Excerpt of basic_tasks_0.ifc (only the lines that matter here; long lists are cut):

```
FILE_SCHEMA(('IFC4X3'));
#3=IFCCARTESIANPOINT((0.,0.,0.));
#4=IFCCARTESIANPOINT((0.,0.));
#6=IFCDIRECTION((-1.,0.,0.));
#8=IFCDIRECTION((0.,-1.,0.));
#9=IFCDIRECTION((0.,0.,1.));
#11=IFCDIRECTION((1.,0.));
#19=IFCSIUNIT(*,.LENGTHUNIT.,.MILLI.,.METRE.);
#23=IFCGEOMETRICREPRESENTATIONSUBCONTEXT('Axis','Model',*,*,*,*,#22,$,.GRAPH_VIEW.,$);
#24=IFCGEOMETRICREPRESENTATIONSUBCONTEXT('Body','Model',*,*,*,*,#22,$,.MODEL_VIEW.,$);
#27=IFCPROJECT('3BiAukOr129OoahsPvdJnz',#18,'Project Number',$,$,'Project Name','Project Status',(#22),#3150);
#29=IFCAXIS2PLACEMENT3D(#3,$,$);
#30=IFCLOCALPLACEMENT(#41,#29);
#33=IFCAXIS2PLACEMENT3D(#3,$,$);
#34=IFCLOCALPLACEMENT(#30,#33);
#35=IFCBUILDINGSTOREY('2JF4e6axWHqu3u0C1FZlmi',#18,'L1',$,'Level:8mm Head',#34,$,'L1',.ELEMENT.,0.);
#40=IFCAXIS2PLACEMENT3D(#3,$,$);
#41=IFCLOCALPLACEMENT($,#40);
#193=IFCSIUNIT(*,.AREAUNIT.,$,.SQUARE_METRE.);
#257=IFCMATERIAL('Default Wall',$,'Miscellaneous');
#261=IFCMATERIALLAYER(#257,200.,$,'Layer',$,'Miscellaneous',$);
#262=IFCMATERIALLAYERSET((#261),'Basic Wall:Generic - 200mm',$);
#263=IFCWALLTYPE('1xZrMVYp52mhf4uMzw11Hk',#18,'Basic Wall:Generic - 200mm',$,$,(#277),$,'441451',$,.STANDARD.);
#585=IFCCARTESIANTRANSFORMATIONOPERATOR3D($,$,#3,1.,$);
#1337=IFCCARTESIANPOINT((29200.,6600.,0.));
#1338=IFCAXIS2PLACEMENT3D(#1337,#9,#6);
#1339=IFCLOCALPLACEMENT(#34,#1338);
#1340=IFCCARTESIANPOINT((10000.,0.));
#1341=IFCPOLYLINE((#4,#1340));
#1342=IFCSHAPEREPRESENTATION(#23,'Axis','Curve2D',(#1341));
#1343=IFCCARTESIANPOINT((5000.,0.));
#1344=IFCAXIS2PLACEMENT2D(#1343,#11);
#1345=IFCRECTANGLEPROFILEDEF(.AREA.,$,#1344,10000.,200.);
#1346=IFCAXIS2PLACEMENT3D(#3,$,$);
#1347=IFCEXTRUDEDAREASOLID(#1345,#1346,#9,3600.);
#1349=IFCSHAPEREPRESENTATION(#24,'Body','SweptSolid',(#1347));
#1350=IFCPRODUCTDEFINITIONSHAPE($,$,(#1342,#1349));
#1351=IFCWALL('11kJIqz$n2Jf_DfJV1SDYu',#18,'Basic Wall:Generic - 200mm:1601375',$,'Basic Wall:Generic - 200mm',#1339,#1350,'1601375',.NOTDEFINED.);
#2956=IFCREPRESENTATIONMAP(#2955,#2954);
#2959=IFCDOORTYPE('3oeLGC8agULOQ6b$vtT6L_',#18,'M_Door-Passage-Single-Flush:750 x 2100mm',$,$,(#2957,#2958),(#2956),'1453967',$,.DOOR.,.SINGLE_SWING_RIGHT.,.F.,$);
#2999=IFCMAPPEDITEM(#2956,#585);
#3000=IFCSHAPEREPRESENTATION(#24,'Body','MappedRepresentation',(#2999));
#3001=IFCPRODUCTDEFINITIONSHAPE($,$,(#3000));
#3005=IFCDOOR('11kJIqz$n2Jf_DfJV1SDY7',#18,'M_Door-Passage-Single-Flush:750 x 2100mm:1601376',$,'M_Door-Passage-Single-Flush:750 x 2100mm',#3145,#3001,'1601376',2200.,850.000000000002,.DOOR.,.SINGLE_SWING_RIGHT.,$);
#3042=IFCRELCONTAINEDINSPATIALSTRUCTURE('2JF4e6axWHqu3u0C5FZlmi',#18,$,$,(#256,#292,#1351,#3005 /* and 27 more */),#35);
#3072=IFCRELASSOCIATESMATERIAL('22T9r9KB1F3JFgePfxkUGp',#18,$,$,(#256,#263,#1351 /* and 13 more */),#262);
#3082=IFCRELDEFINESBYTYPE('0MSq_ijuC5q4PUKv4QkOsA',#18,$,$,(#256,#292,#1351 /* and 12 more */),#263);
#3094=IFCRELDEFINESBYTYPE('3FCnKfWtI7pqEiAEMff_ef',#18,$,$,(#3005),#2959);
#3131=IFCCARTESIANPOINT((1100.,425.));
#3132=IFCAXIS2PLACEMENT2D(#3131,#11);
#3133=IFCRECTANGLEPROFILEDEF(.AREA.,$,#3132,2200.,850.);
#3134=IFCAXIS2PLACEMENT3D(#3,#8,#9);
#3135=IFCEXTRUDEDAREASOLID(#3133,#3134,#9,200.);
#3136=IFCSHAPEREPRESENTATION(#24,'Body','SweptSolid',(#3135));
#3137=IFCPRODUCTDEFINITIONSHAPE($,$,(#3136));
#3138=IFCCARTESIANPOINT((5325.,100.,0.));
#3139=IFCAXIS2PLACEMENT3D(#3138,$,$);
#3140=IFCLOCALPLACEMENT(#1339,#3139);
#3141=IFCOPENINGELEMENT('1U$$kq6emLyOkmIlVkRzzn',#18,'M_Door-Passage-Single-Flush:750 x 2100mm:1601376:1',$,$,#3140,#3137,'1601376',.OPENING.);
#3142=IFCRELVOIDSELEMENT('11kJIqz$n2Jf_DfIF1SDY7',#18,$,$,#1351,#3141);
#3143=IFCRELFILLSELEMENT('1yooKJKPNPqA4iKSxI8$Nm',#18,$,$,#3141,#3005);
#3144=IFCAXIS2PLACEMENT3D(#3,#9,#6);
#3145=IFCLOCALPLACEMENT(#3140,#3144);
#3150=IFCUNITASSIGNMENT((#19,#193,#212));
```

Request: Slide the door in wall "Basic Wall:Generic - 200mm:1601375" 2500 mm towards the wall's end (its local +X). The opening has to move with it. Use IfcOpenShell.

```python
import ifcopenshell
import ifcopenshell.api.geometry
import ifcopenshell.util.placement
import ifcopenshell.util.unit

model = ifcopenshell.open("basic_tasks_0.ifc")
unit_scale = ifcopenshell.util.unit.calculate_unit_scale(model)

door = model.by_guid("11kJIqz$n2Jf_DfJV1SDY7")
opening = door.FillsVoids[0].RelatingOpeningElement
wall = opening.VoidsElements[0].RelatingBuildingElement

wall_matrix = ifcopenshell.util.placement.get_local_placement(wall.ObjectPlacement)
shift = wall_matrix[:3, 0] * 2.5 / unit_scale
before = ifcopenshell.util.placement.get_local_placement(door.ObjectPlacement)[:3, 3].copy()

# The door is placed relative to its opening, so it follows when the opening moves.
matrix = ifcopenshell.util.placement.get_local_placement(opening.ObjectPlacement)
matrix[:3, 3] += shift
ifcopenshell.api.geometry.edit_object_placement(
    model, product=opening, matrix=matrix, is_si=False, should_transform_children=True
)

after = ifcopenshell.util.placement.get_local_placement(door.ObjectPlacement)[:3, 3]
print("door moved by", (after - before).round(3) + 0.0)

model.write("basic_tasks_0-out.ifc")
```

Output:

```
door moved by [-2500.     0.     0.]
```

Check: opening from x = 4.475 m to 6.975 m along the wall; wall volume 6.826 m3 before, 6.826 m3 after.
